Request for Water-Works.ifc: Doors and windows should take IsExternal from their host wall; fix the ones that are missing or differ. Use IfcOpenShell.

First a look at what the model holds.

```python
import ifcopenshell
import ifcopenshell.util.element

model = ifcopenshell.open("Water-Works.ifc")
print(model.schema)
seen = {}
for e in model.by_type("IfcDoor") + model.by_type("IfcWindow"):
    if not e.FillsVoids:
        continue
    host = e.FillsVoids[0].RelatingOpeningElement.VoidsElements[0].RelatingBuildingElement
    own = ifcopenshell.util.element.get_pset(e, f"Pset_{e.is_a()[3:].removesuffix('StandardCase')}Common", "IsExternal")
    wall = ifcopenshell.util.element.get_pset(host, "Pset_WallCommon", "IsExternal")
    seen[e.is_a(), own, wall] = seen.get((e.is_a(), own, wall), 0) + 1
for (cls, own, wall), count in sorted(seen.items(), key=str):
    print(count, cls, "IsExternal:", own, "| host wall:", wall)
```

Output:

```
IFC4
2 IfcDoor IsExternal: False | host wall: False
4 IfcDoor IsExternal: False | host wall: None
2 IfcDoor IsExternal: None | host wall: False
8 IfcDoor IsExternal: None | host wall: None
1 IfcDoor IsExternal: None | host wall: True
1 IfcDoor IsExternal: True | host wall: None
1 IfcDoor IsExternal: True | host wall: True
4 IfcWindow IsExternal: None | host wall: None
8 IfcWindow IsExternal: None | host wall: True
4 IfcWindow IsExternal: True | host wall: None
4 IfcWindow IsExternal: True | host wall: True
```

```python
import ifcopenshell
import ifcopenshell.api.pset
import ifcopenshell.util.element

model = ifcopenshell.open("Water-Works.ifc")

count = 0
for ifc_class, pset_name in (("IfcDoor", "Pset_DoorCommon"), ("IfcWindow", "Pset_WindowCommon")):
    for e in model.by_type(ifc_class):
        if not e.FillsVoids:
            continue
        host = e.FillsVoids[0].RelatingOpeningElement.VoidsElements[0].RelatingBuildingElement
        external = ifcopenshell.util.element.get_pset(host, "Pset_WallCommon", "IsExternal")
        if external is None or ifcopenshell.util.element.get_pset(e, pset_name, "IsExternal") == external:
            continue
        pset = ifcopenshell.api.pset.add_pset(model, product=e, name=pset_name)
        ifcopenshell.api.pset.edit_pset(model, pset=pset, properties={"IsExternal": external})
        count += 1

print(count, "updated")

model.write("Water-Works_updated.ifc")
```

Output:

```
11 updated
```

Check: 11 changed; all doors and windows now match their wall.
